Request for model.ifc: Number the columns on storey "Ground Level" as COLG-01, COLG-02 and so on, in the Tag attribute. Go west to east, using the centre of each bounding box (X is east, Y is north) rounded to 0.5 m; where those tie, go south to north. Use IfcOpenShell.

First a look at what the model holds.

```python
import ifcopenshell
import ifcopenshell.util.element
import ifcopenshell.util.placement

model = ifcopenshell.open("model.ifc")
print(model.schema)
storey = next(s for s in model.by_type("IfcBuildingStorey") if s.Name == "Ground Level")
columns = [e for e in ifcopenshell.util.element.get_decomposition(storey) if e.is_a("IfcColumn")]
for e in sorted(columns, key=lambda e: e.id()):
    origin = ifcopenshell.util.placement.get_local_placement(e.ObjectPlacement)[:3, 3]
    print(e.id(), e.Tag, e.Name, origin.round(2) + 0.0, sep=" | ")
```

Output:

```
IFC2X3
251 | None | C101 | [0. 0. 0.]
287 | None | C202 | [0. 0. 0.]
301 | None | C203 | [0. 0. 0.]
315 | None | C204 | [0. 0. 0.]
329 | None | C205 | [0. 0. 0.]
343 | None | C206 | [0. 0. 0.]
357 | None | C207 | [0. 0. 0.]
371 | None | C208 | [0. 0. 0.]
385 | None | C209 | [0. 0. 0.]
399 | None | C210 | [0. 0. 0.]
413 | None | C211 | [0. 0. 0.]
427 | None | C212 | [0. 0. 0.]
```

```python
import ifcopenshell
import ifcopenshell.geom
import ifcopenshell.util.element
import ifcopenshell.util.shape

model = ifcopenshell.open("model.ifc")
settings = ifcopenshell.geom.settings()
settings.set("use-world-coords", True)


def centre(element):
    shape = ifcopenshell.geom.create_shape(settings, element)
    return ifcopenshell.util.shape.get_bbox_centroid(shape.geometry)


storey = next(s for s in model.by_type("IfcBuildingStorey") if s.Name == "Ground Level")
columns = [e for e in ifcopenshell.util.element.get_decomposition(storey) if e.is_a("IfcColumn")]

# Insertion points can sit at a corner or the storey origin, so sort by the geometry (in metres).
centres = {e: centre(e) for e in columns}
columns.sort(key=lambda e: (round(centres[e][0] / 0.5), centres[e][1]))

for i, e in enumerate(columns, start=1):
    number = f"COLG-{i:02d}"
    e.Tag = number
    print(e.id(), number)

model.write("model_updated.ifc")
```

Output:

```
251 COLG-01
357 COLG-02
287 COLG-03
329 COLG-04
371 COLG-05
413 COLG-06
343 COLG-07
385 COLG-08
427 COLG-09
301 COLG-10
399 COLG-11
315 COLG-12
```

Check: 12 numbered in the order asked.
